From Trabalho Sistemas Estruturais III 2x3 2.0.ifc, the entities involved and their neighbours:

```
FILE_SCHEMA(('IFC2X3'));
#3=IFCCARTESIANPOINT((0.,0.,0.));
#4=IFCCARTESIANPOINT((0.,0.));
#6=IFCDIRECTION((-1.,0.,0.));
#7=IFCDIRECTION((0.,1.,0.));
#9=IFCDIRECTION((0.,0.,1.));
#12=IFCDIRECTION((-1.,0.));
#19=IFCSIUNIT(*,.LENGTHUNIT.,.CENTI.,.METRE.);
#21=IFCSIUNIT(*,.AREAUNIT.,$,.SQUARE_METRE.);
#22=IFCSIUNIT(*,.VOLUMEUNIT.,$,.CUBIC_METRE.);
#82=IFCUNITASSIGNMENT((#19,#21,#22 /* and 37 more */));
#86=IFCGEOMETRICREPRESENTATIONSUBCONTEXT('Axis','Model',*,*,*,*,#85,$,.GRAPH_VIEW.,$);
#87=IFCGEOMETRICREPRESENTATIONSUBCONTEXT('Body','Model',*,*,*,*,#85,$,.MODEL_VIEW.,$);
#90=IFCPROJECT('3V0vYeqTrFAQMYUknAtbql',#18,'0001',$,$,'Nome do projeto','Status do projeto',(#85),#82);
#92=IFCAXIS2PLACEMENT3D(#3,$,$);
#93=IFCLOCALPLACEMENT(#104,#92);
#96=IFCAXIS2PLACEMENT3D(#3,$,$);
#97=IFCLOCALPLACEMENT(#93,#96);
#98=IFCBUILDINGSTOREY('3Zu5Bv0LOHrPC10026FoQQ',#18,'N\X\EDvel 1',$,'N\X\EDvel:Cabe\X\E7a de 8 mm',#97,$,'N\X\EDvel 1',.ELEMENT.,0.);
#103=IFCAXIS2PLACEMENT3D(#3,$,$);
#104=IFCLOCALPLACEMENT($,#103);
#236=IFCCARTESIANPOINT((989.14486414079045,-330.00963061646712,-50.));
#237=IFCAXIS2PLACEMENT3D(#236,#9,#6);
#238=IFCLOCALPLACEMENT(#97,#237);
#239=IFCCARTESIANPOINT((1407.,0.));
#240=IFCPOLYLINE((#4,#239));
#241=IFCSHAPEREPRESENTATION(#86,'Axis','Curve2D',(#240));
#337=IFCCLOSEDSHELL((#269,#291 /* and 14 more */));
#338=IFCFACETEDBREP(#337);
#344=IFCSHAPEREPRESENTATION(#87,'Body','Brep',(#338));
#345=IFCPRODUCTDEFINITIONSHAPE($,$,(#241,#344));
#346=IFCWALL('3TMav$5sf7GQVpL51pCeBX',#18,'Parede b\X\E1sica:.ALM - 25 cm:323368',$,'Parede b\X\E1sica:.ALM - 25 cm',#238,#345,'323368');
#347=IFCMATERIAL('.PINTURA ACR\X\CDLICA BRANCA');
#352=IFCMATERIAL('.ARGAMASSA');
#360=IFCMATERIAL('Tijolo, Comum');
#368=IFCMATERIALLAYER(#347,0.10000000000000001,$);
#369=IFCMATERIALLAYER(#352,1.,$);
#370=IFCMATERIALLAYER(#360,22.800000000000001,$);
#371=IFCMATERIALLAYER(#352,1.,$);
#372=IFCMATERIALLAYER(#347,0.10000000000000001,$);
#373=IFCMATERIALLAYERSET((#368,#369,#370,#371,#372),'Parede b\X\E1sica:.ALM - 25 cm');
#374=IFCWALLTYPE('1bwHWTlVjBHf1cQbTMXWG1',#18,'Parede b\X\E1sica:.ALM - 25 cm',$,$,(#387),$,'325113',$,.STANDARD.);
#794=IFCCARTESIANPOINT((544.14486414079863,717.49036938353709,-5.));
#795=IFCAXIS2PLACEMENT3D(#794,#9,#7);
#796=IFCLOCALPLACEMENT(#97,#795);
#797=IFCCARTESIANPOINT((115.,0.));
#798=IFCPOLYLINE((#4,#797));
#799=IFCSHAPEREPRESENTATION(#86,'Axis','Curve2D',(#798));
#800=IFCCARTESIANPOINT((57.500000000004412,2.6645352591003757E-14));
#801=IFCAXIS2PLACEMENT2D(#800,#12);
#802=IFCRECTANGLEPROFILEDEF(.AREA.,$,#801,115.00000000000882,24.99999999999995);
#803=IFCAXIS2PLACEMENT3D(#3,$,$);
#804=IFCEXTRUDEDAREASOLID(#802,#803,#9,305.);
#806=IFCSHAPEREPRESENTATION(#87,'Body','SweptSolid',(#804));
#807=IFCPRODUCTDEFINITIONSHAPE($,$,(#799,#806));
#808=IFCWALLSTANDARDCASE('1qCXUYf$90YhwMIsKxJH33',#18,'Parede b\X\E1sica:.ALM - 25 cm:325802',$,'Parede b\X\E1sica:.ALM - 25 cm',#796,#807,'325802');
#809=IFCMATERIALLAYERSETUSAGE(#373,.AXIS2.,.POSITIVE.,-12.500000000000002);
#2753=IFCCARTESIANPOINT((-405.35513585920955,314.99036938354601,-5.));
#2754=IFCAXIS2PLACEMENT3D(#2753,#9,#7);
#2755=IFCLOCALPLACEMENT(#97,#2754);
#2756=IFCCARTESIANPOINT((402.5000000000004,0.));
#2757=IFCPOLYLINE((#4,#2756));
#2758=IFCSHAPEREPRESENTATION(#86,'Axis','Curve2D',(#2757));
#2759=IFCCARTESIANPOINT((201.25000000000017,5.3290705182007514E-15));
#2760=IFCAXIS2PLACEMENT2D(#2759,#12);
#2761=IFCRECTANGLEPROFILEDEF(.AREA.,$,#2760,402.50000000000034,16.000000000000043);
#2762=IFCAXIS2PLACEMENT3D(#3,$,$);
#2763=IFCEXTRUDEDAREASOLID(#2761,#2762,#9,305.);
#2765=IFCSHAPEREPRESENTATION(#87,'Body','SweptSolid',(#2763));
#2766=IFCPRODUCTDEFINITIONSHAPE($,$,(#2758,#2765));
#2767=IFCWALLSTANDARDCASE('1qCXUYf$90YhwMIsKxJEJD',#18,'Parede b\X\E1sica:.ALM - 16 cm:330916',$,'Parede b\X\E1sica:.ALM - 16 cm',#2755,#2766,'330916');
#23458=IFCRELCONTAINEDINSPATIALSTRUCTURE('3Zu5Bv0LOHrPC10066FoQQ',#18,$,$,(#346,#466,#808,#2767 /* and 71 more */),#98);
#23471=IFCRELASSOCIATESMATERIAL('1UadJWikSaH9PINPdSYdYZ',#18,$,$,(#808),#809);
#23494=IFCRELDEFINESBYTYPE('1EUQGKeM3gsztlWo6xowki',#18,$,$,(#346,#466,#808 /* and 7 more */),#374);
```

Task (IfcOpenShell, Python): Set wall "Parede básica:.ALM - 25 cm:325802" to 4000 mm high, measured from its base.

```python
import ifcopenshell
import ifcopenshell.geom
import ifcopenshell.util.representation
import ifcopenshell.util.shape
import ifcopenshell.util.unit

model = ifcopenshell.open("Trabalho Sistemas Estruturais III 2x3 2.0.ifc")
unit_scale = ifcopenshell.util.unit.calculate_unit_scale(model)
settings = ifcopenshell.geom.settings()


def volume(element):
    """Net volume in cubic metres, openings subtracted."""
    shape = ifcopenshell.geom.create_shape(settings, element)
    return ifcopenshell.util.shape.get_volume(shape.geometry)


wall = model.by_id(808)
before = volume(wall)

body = ifcopenshell.util.representation.get_representation(wall, "Model", "Body")
solid = body.Items[0]
old_height = solid.Depth
solid.Depth = 4 / unit_scale
after = volume(wall)

print(f"height {old_height:g} -> {solid.Depth:g}, volume {before:.3f} -> {after:.3f} m3")

model.write("Trabalho Sistemas Estruturais III 2x3 2.0_rev.ifc")
```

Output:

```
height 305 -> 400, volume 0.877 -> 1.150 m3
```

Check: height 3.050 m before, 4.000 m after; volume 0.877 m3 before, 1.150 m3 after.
